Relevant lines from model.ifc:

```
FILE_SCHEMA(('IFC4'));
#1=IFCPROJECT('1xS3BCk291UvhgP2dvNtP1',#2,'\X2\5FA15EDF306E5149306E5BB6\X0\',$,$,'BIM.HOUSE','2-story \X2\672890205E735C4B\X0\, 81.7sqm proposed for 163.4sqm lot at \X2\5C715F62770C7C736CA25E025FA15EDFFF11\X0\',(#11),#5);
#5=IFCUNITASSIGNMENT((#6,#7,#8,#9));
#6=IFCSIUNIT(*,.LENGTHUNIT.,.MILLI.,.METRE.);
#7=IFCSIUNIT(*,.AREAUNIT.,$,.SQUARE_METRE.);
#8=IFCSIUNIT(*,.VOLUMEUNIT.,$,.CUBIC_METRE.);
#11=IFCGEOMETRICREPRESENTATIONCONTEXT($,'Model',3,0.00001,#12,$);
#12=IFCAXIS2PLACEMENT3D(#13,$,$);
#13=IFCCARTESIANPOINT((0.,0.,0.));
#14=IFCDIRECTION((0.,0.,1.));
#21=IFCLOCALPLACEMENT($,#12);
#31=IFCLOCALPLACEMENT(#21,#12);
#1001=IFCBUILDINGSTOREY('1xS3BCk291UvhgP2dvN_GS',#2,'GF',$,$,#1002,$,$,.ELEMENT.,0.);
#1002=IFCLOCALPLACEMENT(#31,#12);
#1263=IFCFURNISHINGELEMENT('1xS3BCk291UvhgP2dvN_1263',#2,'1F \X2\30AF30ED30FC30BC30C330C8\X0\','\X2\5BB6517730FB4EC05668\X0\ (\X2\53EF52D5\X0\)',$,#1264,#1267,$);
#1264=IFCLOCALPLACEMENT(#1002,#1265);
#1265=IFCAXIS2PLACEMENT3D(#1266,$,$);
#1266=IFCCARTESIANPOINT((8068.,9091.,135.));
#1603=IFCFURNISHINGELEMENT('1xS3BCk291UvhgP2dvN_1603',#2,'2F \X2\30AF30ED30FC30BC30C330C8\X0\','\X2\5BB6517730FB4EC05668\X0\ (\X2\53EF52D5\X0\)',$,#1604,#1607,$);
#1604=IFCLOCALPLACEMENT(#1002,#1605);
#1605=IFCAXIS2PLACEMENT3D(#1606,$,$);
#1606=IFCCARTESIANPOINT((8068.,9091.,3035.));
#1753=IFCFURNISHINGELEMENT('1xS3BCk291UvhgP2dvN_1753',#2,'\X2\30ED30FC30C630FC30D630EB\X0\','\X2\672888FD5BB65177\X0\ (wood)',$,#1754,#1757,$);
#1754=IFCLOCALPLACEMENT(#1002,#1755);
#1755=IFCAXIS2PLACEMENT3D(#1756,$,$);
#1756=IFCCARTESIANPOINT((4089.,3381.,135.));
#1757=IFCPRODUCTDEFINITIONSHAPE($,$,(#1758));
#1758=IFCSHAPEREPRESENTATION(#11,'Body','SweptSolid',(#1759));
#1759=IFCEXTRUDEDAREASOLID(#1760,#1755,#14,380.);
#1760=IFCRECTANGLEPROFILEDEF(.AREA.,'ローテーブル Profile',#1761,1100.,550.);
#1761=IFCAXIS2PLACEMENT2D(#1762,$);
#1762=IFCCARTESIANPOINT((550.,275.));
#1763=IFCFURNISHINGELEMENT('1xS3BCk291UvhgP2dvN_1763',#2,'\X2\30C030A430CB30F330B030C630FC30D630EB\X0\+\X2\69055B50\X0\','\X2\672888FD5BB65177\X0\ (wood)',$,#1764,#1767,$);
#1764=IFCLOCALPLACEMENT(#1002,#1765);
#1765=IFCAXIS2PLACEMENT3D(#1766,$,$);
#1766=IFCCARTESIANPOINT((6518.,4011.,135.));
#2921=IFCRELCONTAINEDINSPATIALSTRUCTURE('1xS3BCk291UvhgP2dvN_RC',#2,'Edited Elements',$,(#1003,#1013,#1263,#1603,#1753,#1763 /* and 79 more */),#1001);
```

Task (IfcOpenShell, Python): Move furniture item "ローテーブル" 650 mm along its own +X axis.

```python
import ifcopenshell
import ifcopenshell.api.geometry
import ifcopenshell.util.placement
import ifcopenshell.util.unit

model = ifcopenshell.open("model.ifc")
unit_scale = ifcopenshell.util.unit.calculate_unit_scale(model)

item = model.by_id(1753)
matrix = ifcopenshell.util.placement.get_local_placement(item.ObjectPlacement)
matrix[:3, 3] += matrix[:3, 0] * 0.65 / unit_scale
ifcopenshell.api.geometry.edit_object_placement(model, product=item, matrix=matrix, is_si=False)

print(ifcopenshell.util.placement.get_local_placement(item.ObjectPlacement).round(3) + 0.0)

model.write("model_rev.ifc")
```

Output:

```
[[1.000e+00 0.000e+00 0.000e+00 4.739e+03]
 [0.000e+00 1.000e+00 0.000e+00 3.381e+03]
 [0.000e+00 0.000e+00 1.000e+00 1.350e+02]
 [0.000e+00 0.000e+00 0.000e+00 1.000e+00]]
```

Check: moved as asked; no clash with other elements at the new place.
